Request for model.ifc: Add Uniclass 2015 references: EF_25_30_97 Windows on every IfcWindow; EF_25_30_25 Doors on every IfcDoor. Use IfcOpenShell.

First a look at what the model holds.

```python
import ifcopenshell

model = ifcopenshell.open("model.ifc")
print(model.schema)
print("classifications:", [c.Name for c in model.by_type("IfcClassification")])
for ifc_class in ("IfcDoor", "IfcRoof", "IfcStair", "IfcWall", "IfcWindow"):
    print(ifc_class, len(model.by_type(ifc_class)))
```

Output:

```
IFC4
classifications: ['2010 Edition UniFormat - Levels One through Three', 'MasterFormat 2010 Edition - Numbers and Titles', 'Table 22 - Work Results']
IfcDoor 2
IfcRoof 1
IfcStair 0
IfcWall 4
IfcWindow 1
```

```python
import ifcopenshell
import ifcopenshell.api.classification

model = ifcopenshell.open("model.ifc")

system = ifcopenshell.api.classification.add_classification(model, classification="Uniclass 2015")

codes = {
    "IfcWindow": ("EF_25_30_97", "Windows"),
    "IfcDoor": ("EF_25_30_25", "Doors"),
}
for ifc_class, (code, name) in codes.items():
    products = model.by_type(ifc_class)
    ifcopenshell.api.classification.add_reference(
        model, products=products, classification=system, identification=code, name=name
    )
    print(code, len(products))

model.write("model_edited.ifc")
```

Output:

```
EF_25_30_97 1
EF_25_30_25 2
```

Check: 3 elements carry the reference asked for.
